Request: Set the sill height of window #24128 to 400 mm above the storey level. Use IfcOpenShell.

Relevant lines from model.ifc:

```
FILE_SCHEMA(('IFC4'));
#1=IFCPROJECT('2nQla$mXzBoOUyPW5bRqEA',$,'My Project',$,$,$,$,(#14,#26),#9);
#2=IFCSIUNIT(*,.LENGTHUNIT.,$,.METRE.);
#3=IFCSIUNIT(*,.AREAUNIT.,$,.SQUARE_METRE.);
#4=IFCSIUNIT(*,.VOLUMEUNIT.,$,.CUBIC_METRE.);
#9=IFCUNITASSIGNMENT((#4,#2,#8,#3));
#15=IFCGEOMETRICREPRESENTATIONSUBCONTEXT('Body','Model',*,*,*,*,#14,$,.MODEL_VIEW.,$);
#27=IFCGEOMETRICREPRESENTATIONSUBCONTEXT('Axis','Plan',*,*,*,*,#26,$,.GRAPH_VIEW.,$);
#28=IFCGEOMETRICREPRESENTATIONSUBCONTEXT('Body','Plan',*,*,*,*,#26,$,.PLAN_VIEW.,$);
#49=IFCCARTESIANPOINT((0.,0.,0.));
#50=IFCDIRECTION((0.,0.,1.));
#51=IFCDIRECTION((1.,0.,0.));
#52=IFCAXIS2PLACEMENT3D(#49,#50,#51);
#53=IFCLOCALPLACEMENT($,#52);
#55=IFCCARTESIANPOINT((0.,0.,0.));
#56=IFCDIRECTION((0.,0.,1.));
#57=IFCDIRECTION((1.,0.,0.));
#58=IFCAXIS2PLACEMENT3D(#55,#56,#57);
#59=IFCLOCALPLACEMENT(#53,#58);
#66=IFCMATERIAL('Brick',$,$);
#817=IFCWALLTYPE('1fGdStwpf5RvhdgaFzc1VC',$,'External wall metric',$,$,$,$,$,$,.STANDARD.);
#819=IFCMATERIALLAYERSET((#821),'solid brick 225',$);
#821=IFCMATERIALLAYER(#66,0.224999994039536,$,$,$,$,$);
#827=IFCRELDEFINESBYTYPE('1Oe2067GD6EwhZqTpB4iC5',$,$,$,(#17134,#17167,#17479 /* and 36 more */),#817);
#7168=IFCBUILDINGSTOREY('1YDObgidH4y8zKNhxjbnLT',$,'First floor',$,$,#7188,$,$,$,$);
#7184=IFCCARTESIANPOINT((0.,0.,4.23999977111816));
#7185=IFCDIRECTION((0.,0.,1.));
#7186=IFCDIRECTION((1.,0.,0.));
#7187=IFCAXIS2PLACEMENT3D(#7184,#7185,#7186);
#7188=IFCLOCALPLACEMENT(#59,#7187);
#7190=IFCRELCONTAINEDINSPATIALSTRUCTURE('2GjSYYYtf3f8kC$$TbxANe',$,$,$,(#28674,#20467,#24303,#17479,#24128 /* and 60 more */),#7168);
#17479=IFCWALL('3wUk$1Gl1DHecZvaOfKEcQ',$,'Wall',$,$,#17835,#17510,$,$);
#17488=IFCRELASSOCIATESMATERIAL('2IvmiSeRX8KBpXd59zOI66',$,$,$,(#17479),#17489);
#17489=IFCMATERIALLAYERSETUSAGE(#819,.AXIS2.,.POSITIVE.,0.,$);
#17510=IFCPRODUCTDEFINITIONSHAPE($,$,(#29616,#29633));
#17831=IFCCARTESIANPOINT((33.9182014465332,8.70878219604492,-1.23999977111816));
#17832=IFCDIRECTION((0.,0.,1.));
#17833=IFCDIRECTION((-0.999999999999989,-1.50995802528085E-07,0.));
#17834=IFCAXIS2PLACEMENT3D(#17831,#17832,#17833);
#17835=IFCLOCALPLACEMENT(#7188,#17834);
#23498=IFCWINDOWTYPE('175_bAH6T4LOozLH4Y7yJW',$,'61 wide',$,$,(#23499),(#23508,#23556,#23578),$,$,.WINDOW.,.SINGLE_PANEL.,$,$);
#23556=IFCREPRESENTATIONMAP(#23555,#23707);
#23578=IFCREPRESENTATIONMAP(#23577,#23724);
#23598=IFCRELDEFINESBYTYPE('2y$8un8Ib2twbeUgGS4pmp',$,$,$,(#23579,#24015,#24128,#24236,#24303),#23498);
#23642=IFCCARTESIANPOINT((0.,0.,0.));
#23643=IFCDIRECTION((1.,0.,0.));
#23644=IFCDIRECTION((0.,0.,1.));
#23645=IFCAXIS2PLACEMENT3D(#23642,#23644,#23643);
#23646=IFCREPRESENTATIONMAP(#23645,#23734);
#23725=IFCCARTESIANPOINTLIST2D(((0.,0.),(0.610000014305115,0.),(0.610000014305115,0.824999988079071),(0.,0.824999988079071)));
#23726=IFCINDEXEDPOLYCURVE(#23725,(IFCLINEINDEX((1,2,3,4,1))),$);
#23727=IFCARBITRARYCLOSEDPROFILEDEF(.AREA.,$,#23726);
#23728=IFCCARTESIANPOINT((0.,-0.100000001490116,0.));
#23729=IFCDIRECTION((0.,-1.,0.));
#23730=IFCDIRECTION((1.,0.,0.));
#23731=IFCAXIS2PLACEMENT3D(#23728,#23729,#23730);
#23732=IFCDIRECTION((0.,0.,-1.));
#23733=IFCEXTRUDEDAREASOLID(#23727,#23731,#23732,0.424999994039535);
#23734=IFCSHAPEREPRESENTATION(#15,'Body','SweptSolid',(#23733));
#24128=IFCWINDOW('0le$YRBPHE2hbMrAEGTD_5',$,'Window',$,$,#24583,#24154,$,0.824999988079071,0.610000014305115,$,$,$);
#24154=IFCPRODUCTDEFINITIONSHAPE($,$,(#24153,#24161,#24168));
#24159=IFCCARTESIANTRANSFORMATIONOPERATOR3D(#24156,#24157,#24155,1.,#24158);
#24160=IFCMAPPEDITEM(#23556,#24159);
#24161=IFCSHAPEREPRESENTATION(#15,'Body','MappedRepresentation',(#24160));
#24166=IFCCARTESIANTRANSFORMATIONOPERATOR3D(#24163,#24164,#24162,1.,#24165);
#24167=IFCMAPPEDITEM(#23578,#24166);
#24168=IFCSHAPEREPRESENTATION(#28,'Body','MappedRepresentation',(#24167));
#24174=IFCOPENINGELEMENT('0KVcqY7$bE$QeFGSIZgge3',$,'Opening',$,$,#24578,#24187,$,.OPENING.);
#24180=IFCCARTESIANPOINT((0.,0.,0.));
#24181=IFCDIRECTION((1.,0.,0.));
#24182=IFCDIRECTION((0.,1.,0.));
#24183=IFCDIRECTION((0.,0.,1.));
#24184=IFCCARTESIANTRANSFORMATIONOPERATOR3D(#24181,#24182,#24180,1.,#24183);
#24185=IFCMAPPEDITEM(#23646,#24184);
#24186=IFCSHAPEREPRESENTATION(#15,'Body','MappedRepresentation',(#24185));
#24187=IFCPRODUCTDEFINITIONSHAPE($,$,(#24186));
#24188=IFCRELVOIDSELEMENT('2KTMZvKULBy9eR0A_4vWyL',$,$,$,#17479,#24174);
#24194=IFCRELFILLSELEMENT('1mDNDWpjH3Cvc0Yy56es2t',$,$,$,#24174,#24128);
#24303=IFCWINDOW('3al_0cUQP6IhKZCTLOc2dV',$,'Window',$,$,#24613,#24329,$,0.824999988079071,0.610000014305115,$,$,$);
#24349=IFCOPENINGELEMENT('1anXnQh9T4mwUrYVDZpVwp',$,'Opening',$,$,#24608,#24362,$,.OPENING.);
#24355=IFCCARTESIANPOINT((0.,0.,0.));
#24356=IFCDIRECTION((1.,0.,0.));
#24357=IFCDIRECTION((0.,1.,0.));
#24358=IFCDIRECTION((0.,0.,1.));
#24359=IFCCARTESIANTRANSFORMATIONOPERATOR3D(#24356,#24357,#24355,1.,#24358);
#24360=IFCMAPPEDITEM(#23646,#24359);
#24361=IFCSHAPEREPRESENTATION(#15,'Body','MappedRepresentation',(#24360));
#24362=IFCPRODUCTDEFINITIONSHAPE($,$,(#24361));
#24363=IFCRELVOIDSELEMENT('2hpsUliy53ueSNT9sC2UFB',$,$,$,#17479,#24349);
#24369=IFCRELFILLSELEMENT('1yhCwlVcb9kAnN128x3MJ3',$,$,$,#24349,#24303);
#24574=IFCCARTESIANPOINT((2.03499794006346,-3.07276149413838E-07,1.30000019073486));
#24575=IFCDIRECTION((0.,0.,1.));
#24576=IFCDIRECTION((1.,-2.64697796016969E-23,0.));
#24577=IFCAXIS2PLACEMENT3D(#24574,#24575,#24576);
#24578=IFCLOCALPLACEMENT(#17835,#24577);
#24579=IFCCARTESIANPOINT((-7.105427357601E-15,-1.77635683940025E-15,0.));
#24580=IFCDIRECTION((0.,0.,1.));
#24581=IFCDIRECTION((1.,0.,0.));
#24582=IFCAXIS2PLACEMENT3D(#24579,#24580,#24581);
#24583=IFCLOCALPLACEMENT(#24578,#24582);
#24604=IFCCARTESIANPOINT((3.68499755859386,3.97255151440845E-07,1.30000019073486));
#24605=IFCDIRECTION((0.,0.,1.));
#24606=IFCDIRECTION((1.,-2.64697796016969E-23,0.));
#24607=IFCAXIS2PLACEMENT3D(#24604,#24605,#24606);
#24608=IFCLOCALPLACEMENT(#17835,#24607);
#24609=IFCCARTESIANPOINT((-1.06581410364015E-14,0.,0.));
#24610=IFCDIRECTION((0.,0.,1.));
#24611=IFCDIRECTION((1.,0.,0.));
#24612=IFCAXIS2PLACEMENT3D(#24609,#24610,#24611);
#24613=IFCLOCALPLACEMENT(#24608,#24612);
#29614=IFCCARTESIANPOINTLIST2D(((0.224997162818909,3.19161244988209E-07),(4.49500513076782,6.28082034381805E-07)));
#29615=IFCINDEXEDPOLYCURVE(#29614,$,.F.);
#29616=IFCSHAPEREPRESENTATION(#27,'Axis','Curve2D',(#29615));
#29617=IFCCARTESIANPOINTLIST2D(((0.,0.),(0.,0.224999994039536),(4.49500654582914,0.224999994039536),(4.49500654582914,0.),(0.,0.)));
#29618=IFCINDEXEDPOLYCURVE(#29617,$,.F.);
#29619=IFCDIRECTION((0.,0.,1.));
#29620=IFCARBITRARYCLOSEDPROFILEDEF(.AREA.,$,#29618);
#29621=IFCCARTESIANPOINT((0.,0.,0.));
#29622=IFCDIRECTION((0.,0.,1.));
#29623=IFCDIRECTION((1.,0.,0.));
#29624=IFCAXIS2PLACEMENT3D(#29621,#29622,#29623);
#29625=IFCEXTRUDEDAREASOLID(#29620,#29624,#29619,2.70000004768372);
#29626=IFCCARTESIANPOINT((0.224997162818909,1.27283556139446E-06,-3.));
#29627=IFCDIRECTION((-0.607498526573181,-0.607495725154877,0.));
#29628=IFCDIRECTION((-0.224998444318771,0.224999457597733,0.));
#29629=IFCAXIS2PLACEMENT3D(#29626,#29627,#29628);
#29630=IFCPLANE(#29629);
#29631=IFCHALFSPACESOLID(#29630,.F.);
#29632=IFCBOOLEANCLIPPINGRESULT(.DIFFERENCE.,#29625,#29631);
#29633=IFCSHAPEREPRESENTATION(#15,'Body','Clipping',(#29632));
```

```python
import numpy as np
import ifcopenshell
import ifcopenshell.api.geometry
import ifcopenshell.geom
import ifcopenshell.util.element
import ifcopenshell.util.placement
import ifcopenshell.util.shape
import ifcopenshell.util.unit

model = ifcopenshell.open("model.ifc")
unit_scale = ifcopenshell.util.unit.calculate_unit_scale(model)

window = model.by_guid("0le$YRBPHE2hbMrAEGTD_5")
opening = window.FillsVoids[0].RelatingOpeningElement
storey = ifcopenshell.util.element.get_container(window, ifc_class="IfcBuildingStorey")
level = ifcopenshell.util.placement.get_local_placement(storey.ObjectPlacement)[2, 3]

# The opening's origin need not be at the sill, so measure its lowest point.
shape = ifcopenshell.geom.create_shape(ifcopenshell.geom.settings(), opening)
bottom = ifcopenshell.util.shape.get_shape_bottom_elevation(shape, shape.geometry) / unit_scale
dz = level + 0.4 - bottom

shift = np.array([0.0, 0.0, dz])
# The window is placed relative to its opening, so it follows when the opening moves.
matrix = ifcopenshell.util.placement.get_local_placement(opening.ObjectPlacement)
matrix[:3, 3] += shift
ifcopenshell.api.geometry.edit_object_placement(
    model, product=opening, matrix=matrix, is_si=False, should_transform_children=True
)

print(f"moved by {dz * unit_scale:+.3f} m")

model.write("model_v2.ifc")
```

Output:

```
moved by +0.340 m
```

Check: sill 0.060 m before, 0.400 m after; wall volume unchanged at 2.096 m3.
